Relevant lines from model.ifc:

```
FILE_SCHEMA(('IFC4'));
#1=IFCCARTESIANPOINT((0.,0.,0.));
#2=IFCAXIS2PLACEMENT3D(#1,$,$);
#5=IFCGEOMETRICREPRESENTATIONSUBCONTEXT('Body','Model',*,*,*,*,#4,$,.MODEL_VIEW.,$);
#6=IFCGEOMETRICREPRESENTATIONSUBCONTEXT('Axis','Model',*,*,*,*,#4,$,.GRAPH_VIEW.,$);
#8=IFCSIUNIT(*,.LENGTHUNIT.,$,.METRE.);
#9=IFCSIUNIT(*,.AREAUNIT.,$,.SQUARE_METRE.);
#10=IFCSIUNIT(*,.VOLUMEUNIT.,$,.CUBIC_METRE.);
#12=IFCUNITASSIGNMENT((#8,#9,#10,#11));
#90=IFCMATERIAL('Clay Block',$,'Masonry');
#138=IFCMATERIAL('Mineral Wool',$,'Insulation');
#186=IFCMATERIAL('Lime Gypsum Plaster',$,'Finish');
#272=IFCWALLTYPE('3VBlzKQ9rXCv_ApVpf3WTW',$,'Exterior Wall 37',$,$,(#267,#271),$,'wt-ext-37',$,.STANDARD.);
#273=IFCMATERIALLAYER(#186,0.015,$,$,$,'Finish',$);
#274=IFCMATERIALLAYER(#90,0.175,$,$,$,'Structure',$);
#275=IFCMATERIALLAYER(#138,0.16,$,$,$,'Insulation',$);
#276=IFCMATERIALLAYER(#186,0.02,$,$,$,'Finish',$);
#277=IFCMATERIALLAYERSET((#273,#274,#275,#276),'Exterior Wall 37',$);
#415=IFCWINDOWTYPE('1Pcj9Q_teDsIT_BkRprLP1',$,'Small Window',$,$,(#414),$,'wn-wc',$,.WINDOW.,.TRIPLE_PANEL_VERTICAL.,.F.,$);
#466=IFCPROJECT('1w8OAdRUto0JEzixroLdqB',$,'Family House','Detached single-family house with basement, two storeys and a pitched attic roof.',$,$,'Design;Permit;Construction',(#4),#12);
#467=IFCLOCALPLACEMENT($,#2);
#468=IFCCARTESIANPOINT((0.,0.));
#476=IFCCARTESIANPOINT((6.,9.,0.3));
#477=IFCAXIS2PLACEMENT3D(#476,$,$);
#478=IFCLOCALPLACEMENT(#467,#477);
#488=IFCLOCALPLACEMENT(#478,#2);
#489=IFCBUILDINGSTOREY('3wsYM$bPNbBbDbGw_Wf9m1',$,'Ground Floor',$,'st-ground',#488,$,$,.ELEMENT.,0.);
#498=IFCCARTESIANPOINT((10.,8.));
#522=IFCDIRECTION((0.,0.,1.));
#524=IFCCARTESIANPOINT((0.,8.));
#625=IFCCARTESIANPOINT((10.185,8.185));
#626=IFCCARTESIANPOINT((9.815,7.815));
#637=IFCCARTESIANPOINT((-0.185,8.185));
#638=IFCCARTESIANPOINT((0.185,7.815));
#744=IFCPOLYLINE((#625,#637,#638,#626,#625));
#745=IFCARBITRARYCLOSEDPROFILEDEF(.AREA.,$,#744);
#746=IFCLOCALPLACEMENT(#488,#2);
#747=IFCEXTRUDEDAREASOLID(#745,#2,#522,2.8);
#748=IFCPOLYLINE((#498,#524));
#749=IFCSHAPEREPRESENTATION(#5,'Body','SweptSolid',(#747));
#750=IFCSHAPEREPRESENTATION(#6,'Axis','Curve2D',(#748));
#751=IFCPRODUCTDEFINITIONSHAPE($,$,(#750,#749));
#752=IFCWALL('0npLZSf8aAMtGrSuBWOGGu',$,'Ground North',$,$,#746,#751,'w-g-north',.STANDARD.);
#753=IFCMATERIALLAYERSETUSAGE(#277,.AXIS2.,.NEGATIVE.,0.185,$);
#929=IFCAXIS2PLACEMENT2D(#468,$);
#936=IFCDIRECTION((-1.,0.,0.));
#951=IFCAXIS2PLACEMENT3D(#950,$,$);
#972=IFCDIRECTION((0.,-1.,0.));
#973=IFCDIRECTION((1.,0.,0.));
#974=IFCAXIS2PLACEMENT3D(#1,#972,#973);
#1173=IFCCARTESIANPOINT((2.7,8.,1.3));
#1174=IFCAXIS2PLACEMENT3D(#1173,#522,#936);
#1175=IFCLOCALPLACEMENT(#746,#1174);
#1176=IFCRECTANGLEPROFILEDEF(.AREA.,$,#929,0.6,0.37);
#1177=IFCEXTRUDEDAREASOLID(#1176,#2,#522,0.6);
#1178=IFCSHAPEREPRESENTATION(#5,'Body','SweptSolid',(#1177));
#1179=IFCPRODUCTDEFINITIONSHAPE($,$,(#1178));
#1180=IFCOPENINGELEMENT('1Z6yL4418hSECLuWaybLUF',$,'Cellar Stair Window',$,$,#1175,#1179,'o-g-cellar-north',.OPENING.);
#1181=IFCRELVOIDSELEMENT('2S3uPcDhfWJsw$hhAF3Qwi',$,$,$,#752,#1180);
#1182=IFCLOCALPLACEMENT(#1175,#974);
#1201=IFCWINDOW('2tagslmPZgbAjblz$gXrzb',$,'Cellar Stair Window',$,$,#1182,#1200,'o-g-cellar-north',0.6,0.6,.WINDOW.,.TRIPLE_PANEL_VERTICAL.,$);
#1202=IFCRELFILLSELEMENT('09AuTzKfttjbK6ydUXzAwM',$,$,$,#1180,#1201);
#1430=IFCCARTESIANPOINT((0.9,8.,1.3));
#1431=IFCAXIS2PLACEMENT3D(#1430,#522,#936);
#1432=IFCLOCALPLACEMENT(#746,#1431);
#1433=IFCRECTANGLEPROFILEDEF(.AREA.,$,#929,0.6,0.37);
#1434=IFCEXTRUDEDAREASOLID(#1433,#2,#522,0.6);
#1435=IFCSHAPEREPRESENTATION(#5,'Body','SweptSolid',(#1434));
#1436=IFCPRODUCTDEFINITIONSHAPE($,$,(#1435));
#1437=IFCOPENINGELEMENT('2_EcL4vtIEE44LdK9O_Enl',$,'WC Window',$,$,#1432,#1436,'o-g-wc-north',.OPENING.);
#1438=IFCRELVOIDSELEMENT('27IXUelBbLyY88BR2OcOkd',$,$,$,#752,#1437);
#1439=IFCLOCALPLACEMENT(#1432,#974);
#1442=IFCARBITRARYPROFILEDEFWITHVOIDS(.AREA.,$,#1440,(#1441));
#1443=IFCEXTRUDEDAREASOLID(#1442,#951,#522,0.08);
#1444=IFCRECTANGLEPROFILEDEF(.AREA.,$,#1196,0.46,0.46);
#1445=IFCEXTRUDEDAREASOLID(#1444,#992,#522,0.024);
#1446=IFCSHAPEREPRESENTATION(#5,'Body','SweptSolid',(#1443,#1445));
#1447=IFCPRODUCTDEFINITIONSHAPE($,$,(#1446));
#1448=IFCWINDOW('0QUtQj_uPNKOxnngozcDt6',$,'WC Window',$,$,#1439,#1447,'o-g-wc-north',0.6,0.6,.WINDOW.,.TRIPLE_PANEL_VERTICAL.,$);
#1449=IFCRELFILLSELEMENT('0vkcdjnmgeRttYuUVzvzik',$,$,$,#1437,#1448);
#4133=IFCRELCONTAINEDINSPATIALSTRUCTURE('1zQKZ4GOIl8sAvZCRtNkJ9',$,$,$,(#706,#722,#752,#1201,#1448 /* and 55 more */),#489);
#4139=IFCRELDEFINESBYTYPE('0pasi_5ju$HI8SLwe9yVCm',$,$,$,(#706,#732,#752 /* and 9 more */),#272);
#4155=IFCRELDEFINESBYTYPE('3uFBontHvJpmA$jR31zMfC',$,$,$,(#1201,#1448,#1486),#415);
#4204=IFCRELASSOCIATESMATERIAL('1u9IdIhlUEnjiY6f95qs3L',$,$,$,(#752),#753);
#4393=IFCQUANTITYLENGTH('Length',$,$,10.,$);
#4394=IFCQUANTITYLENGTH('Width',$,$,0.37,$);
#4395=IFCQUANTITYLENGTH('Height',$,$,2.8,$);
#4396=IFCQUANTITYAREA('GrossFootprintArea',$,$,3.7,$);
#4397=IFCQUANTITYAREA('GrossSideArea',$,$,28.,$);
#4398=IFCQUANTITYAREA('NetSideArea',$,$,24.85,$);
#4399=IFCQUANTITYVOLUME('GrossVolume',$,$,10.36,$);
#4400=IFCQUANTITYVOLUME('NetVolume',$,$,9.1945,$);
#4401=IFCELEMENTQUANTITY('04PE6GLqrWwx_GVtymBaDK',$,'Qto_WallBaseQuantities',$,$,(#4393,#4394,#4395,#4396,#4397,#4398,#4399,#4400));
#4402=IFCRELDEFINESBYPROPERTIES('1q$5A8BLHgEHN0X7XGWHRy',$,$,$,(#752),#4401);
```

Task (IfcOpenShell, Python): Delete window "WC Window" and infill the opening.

```python
import ifcopenshell
import ifcopenshell.api.feature
import ifcopenshell.api.pset
import ifcopenshell.api.root
import ifcopenshell.geom
import ifcopenshell.util.element
import ifcopenshell.util.shape
import ifcopenshell.util.unit

model = ifcopenshell.open("model.ifc")
area_scale = ifcopenshell.util.unit.calculate_unit_scale(model, "AREAUNIT")
volume_scale = ifcopenshell.util.unit.calculate_unit_scale(model, "VOLUMEUNIT")
settings = ifcopenshell.geom.settings()


def volume(element):
    """Net volume in cubic metres, openings subtracted."""
    shape = ifcopenshell.geom.create_shape(settings, element)
    return ifcopenshell.util.shape.get_volume(shape.geometry)


window = model.by_id(1448)
opening = window.FillsVoids[0].RelatingOpeningElement
wall = opening.VoidsElements[0].RelatingBuildingElement
before = volume(wall)

ifcopenshell.api.root.remove_product(model, product=window)
ifcopenshell.api.feature.remove_feature(model, feature=opening)

after = volume(wall)
thickness = 0.37  # wall thickness in metres

# Update the wall's stored quantities.
qto = model.by_id(ifcopenshell.util.element.get_pset(wall, "Qto_WallBaseQuantities", should_inherit=False)["id"])
ifcopenshell.api.pset.edit_qto(model, qto=qto, properties={
    "NetSideArea": after / thickness / area_scale,
    "NetVolume": after / volume_scale,
})

print(f"wall volume {before:.3f} -> {after:.3f} m3")

model.write("model-out.ifc")
```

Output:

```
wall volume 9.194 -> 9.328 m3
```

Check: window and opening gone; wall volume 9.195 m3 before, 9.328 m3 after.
